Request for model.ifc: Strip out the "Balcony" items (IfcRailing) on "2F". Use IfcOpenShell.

First a look at what the model holds.

```python
import ifcopenshell
import ifcopenshell.util.element

model = ifcopenshell.open("model.ifc")
print(model.schema)
storey = next(s for s in model.by_type("IfcBuildingStorey") if s.Name == "2F")
railings = [e for e in ifcopenshell.util.element.get_decomposition(storey) if e.is_a("IfcRailing")]
seen = {}
for e in railings:
    element_type = ifcopenshell.util.element.get_type(e)
    name = element_type.Name if element_type not in (None, e) else None
    seen[name] = seen.get(name, 0) + 1
for name, count in sorted(seen.items(), key=str):
    print(count, "x", name)
```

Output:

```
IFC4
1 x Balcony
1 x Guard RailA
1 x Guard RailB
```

```python
import ifcopenshell
import ifcopenshell.api.root
import ifcopenshell.util.element

model = ifcopenshell.open("model.ifc")

storey = next(s for s in model.by_type("IfcBuildingStorey") if s.Name == "2F")
railings = [e for e in ifcopenshell.util.element.get_decomposition(storey) if e.is_a("IfcRailing")]
targets = [e for e in railings if (t := ifcopenshell.util.element.get_type(e)) not in (None, e) and t.Name == "Balcony"]

for e in targets:
    ifcopenshell.api.root.remove_product(model, product=e)
print(len(targets), "removed")

model.write("model-out.ifc")
```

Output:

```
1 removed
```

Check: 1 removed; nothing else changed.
